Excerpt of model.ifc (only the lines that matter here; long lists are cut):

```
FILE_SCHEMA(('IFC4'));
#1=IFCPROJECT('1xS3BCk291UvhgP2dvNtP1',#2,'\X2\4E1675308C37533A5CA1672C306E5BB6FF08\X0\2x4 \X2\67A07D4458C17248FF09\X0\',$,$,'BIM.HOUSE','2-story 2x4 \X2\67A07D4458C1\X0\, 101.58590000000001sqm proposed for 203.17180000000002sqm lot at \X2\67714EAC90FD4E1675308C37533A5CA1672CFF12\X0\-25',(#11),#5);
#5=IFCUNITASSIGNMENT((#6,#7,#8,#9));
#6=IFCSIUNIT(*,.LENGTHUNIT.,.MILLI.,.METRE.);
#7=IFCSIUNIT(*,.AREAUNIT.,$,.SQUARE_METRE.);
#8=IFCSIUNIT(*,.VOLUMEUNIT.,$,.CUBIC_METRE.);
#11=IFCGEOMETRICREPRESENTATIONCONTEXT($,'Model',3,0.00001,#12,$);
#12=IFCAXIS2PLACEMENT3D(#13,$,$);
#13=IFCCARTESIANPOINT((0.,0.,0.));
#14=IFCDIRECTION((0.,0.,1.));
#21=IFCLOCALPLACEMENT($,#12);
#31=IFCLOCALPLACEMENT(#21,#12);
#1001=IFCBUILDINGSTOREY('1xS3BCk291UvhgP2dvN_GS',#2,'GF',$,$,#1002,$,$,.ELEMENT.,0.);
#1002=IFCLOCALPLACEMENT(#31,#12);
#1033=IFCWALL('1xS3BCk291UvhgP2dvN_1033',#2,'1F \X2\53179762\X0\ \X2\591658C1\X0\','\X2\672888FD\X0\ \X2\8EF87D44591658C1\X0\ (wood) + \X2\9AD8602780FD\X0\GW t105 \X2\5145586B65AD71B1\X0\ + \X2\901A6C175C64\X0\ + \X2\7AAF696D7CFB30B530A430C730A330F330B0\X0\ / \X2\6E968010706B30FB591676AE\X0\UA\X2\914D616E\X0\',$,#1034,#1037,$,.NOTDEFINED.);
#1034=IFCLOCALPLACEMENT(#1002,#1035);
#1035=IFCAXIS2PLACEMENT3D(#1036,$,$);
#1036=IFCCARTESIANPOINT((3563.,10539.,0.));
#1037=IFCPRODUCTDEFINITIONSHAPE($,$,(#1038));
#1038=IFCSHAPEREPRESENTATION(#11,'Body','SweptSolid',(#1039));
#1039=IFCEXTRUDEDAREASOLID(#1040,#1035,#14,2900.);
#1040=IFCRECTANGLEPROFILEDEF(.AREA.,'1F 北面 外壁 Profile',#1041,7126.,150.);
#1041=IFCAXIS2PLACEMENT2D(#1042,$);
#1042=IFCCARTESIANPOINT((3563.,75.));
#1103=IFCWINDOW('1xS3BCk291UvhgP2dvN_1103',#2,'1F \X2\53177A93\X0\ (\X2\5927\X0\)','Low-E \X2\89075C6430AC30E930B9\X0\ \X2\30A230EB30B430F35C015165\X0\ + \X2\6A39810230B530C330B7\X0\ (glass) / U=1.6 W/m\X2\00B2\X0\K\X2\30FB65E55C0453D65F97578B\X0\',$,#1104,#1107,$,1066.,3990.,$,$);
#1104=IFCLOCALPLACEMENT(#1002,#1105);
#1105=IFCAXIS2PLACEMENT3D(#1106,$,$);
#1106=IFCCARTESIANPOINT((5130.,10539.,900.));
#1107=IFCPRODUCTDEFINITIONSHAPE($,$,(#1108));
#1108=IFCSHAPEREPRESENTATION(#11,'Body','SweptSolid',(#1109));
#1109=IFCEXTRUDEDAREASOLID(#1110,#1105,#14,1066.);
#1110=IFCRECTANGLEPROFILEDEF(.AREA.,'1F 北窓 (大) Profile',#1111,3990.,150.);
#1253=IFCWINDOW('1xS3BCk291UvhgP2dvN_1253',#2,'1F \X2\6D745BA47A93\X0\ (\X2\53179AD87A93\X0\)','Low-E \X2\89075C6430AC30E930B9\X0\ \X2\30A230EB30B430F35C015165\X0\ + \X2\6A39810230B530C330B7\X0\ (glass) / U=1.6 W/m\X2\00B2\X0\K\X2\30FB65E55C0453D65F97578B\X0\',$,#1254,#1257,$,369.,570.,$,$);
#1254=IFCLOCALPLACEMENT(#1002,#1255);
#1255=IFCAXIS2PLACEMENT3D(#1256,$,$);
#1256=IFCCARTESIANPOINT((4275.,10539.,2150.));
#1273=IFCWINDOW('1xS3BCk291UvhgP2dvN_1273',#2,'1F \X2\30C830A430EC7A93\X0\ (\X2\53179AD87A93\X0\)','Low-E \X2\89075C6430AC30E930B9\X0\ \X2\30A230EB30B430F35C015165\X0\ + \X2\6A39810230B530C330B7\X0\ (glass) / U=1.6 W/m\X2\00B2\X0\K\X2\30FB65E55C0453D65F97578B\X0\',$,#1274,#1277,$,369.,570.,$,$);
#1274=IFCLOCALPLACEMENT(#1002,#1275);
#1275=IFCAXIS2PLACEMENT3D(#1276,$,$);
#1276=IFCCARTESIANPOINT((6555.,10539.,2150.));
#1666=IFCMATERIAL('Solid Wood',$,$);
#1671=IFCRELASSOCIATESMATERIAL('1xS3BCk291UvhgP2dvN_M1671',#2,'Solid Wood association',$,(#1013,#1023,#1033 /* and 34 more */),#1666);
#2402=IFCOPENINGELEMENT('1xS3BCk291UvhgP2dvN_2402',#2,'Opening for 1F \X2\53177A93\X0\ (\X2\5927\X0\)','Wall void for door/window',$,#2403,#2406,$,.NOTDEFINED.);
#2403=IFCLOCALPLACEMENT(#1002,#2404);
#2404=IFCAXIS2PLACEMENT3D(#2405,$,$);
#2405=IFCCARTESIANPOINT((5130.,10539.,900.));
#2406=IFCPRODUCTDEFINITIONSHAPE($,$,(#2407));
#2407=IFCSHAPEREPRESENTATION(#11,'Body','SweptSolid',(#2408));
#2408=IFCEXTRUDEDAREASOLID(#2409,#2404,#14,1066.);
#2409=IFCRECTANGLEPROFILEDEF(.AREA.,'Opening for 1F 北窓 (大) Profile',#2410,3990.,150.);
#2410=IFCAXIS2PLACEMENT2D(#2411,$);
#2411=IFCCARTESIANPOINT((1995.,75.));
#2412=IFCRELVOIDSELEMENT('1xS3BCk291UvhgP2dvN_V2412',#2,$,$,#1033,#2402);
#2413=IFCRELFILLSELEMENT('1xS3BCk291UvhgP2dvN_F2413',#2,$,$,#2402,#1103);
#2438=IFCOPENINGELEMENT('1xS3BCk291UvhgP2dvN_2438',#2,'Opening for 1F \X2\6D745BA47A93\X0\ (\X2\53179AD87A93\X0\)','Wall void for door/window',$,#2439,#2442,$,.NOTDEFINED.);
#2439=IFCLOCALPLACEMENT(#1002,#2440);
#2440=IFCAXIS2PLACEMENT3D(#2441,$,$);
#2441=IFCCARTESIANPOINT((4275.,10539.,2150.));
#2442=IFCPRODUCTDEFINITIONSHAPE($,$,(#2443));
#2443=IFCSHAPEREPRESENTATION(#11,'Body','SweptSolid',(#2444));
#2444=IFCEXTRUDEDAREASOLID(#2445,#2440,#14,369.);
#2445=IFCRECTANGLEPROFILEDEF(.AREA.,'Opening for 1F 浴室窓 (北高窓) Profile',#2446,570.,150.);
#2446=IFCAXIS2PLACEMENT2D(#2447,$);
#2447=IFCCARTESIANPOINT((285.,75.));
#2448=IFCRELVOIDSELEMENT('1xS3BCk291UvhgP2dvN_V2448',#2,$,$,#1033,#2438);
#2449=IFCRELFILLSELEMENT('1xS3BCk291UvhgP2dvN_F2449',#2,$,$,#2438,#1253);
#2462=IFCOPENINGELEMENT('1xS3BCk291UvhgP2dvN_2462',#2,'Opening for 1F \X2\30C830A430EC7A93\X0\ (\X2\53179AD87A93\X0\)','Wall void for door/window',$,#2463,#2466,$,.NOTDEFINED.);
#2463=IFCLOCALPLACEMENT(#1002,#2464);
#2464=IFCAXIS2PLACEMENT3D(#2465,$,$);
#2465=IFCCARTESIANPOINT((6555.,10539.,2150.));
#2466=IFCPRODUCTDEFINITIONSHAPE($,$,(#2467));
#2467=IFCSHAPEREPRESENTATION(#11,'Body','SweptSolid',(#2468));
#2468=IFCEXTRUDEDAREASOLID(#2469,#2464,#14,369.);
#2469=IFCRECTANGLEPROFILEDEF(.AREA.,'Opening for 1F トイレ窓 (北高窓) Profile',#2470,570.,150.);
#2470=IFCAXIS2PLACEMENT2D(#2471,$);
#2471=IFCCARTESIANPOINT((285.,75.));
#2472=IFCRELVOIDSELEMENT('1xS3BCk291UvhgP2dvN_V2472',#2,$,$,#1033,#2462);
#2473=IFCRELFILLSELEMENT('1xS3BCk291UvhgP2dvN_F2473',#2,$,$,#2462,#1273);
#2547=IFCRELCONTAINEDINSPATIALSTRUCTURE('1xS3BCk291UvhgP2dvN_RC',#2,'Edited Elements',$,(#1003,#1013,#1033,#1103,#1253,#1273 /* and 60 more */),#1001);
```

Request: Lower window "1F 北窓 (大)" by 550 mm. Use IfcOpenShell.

```python
import numpy as np
import ifcopenshell
import ifcopenshell.api.geometry
import ifcopenshell.util.placement
import ifcopenshell.util.unit

model = ifcopenshell.open("model.ifc")
unit_scale = ifcopenshell.util.unit.calculate_unit_scale(model)

window = model.by_guid("1xS3BCk291UvhgP2dvN_1103")
opening = window.FillsVoids[0].RelatingOpeningElement
dz = -0.55 / unit_scale

shift = np.array([0.0, 0.0, dz])
# The window is not placed relative to its opening, so move both.
for product in (opening, window):
    matrix = ifcopenshell.util.placement.get_local_placement(product.ObjectPlacement)
    matrix[:3, 3] += shift
    ifcopenshell.api.geometry.edit_object_placement(model, product=product, matrix=matrix, is_si=False)

print(f"moved by {dz * unit_scale:+.3f} m")

model.write("model-out.ifc")
```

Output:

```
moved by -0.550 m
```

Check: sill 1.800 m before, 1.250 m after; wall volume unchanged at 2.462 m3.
